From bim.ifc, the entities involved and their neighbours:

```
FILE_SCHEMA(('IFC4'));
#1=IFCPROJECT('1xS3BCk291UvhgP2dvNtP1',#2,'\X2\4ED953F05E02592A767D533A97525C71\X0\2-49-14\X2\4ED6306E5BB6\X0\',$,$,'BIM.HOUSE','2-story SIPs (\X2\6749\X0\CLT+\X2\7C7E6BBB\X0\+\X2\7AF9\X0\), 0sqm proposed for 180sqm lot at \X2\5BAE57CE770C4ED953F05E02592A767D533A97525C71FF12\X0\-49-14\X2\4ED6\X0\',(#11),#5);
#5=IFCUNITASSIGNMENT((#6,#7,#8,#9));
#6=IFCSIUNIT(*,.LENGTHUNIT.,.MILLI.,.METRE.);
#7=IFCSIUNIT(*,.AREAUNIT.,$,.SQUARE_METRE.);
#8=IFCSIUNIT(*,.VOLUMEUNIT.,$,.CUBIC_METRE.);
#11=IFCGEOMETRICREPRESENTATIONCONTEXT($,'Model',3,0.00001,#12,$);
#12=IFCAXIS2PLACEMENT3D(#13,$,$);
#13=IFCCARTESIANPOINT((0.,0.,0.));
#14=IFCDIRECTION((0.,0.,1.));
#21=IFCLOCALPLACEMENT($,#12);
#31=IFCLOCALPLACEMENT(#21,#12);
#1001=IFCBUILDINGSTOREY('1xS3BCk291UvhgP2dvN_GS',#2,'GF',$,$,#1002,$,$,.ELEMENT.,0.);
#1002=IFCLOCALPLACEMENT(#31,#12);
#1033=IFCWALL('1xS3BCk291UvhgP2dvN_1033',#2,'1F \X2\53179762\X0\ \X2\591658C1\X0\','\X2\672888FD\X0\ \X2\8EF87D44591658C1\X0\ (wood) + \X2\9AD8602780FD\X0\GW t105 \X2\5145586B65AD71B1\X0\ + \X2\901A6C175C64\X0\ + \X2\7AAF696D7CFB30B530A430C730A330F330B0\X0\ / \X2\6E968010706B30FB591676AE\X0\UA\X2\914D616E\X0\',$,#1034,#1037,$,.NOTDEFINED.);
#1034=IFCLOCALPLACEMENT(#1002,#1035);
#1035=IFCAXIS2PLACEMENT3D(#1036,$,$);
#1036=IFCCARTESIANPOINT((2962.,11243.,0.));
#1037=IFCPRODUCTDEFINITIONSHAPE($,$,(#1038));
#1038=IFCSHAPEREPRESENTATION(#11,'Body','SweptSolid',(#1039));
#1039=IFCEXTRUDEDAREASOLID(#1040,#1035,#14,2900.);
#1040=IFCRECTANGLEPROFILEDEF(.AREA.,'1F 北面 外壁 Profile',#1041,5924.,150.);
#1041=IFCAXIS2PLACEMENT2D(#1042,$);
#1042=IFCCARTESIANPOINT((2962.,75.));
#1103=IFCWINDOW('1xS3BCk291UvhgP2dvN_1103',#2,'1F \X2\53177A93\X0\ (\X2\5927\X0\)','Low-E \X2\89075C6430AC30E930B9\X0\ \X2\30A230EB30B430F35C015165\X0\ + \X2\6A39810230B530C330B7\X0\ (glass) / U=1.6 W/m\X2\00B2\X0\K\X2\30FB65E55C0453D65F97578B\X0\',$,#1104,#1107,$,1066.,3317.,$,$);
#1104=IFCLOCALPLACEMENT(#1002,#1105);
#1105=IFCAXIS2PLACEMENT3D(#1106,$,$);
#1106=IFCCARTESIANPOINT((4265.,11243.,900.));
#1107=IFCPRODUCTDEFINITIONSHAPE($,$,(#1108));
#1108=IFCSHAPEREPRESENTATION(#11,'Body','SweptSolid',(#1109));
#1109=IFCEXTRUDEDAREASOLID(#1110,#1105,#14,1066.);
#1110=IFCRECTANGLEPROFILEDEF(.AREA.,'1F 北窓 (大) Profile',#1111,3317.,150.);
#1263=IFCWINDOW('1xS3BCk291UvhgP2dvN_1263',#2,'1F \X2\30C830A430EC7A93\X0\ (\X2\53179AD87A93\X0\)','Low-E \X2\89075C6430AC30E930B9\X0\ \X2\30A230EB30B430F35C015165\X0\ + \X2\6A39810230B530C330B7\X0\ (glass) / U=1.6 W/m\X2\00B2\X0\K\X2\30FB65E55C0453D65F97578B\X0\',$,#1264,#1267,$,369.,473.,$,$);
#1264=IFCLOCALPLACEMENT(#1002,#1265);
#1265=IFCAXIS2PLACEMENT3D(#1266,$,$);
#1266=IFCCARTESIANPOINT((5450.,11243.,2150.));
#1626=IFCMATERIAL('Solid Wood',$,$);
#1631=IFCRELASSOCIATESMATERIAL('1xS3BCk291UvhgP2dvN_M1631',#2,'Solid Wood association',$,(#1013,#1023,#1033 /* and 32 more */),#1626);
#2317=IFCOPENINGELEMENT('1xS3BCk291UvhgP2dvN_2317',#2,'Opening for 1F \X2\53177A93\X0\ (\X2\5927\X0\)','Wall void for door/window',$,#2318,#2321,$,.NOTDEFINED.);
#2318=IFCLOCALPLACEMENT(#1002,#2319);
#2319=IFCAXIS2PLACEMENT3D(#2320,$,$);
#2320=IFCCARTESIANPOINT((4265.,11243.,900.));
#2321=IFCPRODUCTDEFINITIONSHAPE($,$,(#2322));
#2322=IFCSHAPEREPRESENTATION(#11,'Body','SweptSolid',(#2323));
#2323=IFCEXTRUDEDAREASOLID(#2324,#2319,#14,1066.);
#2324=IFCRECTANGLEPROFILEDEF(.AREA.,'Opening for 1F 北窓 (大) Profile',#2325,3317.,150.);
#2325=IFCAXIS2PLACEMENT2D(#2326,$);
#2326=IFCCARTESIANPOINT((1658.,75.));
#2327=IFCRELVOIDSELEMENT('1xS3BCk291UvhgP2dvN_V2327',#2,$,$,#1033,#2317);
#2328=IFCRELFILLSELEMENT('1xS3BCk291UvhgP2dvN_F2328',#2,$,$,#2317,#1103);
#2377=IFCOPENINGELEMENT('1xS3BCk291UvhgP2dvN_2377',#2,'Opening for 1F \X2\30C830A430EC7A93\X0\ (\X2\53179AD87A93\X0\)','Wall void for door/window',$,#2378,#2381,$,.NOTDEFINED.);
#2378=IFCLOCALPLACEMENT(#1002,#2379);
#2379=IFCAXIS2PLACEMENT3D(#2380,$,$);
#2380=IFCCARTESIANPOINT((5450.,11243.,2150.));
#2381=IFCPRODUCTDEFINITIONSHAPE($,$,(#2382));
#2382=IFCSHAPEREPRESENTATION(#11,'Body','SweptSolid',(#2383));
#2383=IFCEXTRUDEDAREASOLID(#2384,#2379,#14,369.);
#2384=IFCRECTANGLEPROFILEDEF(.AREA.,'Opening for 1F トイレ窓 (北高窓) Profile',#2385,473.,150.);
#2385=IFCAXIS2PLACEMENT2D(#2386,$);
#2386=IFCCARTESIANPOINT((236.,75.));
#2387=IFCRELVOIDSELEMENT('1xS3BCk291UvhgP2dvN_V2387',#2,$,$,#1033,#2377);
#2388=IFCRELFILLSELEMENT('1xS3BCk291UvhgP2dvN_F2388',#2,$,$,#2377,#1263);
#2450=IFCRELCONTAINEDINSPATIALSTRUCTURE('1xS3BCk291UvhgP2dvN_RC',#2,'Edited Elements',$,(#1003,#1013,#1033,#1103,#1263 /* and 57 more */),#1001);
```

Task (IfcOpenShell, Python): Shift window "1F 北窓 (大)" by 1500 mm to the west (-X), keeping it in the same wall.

```python
import ifcopenshell
import ifcopenshell.api.geometry
import ifcopenshell.util.placement
import ifcopenshell.util.unit

model = ifcopenshell.open("bim.ifc")
unit_scale = ifcopenshell.util.unit.calculate_unit_scale(model)

window = model.by_guid("1xS3BCk291UvhgP2dvN_1103")
opening = window.FillsVoids[0].RelatingOpeningElement
wall = opening.VoidsElements[0].RelatingBuildingElement

wall_matrix = ifcopenshell.util.placement.get_local_placement(wall.ObjectPlacement)
shift = wall_matrix[:3, 0] * -1.5 / unit_scale
before = ifcopenshell.util.placement.get_local_placement(window.ObjectPlacement)[:3, 3].copy()

# The window is not placed relative to its opening, so move both.
for product in (opening, window):
    matrix = ifcopenshell.util.placement.get_local_placement(product.ObjectPlacement)
    matrix[:3, 3] += shift
    ifcopenshell.api.geometry.edit_object_placement(model, product=product, matrix=matrix, is_si=False)

after = ifcopenshell.util.placement.get_local_placement(window.ObjectPlacement)[:3, 3]
print("window moved by", (after - before).round(3) + 0.0)

model.write("bim_edited.ifc")
```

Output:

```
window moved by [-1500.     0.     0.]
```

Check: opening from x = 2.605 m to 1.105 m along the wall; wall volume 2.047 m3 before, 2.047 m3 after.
